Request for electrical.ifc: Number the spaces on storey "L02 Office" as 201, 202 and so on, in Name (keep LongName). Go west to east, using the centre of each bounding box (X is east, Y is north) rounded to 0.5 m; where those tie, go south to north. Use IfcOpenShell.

First a look at what the model holds.

```python
import ifcopenshell
import ifcopenshell.util.element
import ifcopenshell.util.placement

model = ifcopenshell.open("electrical.ifc")
print(model.schema)
storey = next(s for s in model.by_type("IfcBuildingStorey") if s.Name == "L02 Office")
spaces = [e for e in ifcopenshell.util.element.get_decomposition(storey) if e.is_a("IfcSpace")]
for e in sorted(spaces, key=lambda e: e.id()):
    origin = ifcopenshell.util.placement.get_local_placement(e.ObjectPlacement)[:3, 3]
    print(e.id(), e.Name, e.LongName, origin.round(2) + 0.0, sep=" | ")
```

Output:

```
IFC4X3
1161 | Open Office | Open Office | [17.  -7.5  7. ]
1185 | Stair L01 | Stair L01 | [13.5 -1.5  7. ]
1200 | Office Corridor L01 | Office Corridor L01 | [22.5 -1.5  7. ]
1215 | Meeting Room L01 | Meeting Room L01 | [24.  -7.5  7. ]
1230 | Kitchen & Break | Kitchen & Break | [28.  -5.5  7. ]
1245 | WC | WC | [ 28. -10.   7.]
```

```python
import ifcopenshell
import ifcopenshell.geom
import ifcopenshell.util.element
import ifcopenshell.util.shape

model = ifcopenshell.open("electrical.ifc")
settings = ifcopenshell.geom.settings()
settings.set("use-world-coords", True)


def centre(element):
    shape = ifcopenshell.geom.create_shape(settings, element)
    return ifcopenshell.util.shape.get_bbox_centroid(shape.geometry)


storey = next(s for s in model.by_type("IfcBuildingStorey") if s.Name == "L02 Office")
spaces = [e for e in ifcopenshell.util.element.get_decomposition(storey) if e.is_a("IfcSpace")]

# Insertion points can sit at a corner or the storey origin, so sort by the geometry (in metres).
centres = {e: centre(e) for e in spaces}
spaces.sort(key=lambda e: (round(centres[e][0] / 0.5), centres[e][1]))

for i, e in enumerate(spaces, start=1):
    number = f"2{i:02d}"
    e.Name = number
    print(e.id(), number)

model.write("electrical_edited.ifc")
```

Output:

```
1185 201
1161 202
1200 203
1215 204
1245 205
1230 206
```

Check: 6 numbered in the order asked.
